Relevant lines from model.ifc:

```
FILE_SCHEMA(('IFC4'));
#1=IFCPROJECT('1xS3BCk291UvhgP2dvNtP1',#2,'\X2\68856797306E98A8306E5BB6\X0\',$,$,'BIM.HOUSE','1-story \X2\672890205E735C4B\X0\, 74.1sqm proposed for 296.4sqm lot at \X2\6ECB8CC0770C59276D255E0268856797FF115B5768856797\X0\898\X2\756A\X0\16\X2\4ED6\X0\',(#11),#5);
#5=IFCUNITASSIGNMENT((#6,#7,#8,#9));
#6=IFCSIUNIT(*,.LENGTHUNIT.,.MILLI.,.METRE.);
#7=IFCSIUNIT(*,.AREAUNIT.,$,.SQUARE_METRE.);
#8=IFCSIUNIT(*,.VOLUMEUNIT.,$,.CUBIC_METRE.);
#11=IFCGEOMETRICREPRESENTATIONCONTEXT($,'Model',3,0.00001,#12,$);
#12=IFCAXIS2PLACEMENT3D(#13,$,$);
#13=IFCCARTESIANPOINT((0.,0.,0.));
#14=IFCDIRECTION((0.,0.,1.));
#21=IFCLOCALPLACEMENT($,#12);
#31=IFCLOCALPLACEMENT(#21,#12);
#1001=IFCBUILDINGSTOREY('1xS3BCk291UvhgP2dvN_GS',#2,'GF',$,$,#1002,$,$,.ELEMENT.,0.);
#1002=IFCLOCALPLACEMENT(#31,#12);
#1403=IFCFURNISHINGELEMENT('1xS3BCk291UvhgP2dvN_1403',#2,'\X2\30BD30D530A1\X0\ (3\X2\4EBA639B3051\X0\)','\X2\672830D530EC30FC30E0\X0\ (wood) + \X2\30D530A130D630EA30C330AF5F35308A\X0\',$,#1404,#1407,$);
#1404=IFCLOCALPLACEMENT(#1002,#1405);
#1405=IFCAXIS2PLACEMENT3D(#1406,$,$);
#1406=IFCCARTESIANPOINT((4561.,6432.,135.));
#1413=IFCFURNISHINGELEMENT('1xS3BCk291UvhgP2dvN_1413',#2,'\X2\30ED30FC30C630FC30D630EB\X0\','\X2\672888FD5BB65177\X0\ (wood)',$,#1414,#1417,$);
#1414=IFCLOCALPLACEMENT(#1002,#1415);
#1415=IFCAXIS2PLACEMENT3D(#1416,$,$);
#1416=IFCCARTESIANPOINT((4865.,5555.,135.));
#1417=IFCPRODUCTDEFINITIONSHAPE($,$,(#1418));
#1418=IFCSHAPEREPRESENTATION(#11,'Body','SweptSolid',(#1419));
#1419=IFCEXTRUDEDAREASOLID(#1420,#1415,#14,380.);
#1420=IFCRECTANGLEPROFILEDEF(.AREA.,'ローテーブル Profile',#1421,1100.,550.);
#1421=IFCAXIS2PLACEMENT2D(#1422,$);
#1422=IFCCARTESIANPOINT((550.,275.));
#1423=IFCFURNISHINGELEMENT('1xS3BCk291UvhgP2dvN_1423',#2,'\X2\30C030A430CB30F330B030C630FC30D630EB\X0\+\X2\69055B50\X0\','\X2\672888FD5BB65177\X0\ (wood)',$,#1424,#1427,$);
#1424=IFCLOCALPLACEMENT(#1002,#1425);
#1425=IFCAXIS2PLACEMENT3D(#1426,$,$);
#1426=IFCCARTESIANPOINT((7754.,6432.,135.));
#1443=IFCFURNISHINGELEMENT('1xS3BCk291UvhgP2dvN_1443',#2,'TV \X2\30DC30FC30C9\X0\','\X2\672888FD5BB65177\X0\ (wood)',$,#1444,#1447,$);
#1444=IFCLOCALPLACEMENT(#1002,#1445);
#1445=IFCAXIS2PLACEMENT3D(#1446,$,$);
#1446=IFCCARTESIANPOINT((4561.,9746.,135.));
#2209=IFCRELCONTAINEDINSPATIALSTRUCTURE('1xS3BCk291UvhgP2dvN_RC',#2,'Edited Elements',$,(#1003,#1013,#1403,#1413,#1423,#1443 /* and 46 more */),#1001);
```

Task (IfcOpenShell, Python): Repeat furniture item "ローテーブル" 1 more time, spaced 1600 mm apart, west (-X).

```python
import numpy as np
import ifcopenshell
import ifcopenshell.api.geometry
import ifcopenshell.api.root
import ifcopenshell.util.element
import ifcopenshell.util.placement

model = ifcopenshell.open("model.ifc")


def reuse_history(source, copy):
    """copy_class also copies each property set's owner history, people and application; keep the originals."""
    for rel in copy.IsDefinedBy:
        if rel.is_a("IfcRelDefinesByProperties") and (history := rel.RelatingPropertyDefinition.OwnerHistory):
            rel.RelatingPropertyDefinition.OwnerHistory = source.OwnerHistory
            ifcopenshell.util.element.remove_deep2(model, history)


source = model.by_guid("1xS3BCk291UvhgP2dvN_1413")
base = ifcopenshell.util.placement.get_local_placement(source.ObjectPlacement)
step = np.array([-1.0, 0.0, 0.0]) * 1600.0

for i in range(1, 2):
    copy = ifcopenshell.api.root.copy_class(model, product=source)
    copy.Representation = ifcopenshell.util.element.copy_deep(
        model, source.Representation, exclude=["IfcGeometricRepresentationContext", "IfcRepresentationMap"]
    )
    reuse_history(source, copy)
    matrix = base.copy()
    matrix[:3, 3] += i * step
    print("added at", matrix[:3, 3].round(3) + 0.0)
    ifcopenshell.api.geometry.edit_object_placement(model, product=copy, matrix=matrix, is_si=False)

model.write("model_v2.ifc")
```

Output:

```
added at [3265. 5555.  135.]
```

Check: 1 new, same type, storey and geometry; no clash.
